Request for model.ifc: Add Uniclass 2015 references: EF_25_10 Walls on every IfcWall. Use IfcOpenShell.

First a look at what the model holds.

```python
import ifcopenshell

model = ifcopenshell.open("model.ifc")
print(model.schema)
print("classifications:", [c.Name for c in model.by_type("IfcClassification")])
for ifc_class in ("IfcDoor", "IfcRoof", "IfcStair", "IfcWall", "IfcWindow"):
    print(ifc_class, len(model.by_type(ifc_class)))
```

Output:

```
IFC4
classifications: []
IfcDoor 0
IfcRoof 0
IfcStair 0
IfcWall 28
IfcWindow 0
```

```python
import ifcopenshell
import ifcopenshell.api.classification

model = ifcopenshell.open("model.ifc")

system = ifcopenshell.api.classification.add_classification(model, classification="Uniclass 2015")

codes = {
    "IfcWall": ("EF_25_10", "Walls"),
}
for ifc_class, (code, name) in codes.items():
    products = model.by_type(ifc_class)
    ifcopenshell.api.classification.add_reference(
        model, products=products, classification=system, identification=code, name=name
    )
    print(code, len(products))

model.write("model_edited.ifc")
```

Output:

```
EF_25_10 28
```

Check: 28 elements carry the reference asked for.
